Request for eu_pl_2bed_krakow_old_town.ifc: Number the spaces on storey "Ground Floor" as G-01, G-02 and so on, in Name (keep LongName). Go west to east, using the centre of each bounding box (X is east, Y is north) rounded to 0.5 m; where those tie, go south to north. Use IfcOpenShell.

First a look at what the model holds.

```python
import ifcopenshell
import ifcopenshell.util.element
import ifcopenshell.util.placement

model = ifcopenshell.open("eu_pl_2bed_krakow_old_town.ifc")
print(model.schema)
storey = next(s for s in model.by_type("IfcBuildingStorey") if s.Name == "Ground Floor")
spaces = [e for e in ifcopenshell.util.element.get_decomposition(storey) if e.is_a("IfcSpace")]
for e in sorted(spaces, key=lambda e: e.id()):
    origin = ifcopenshell.util.placement.get_local_placement(e.ObjectPlacement)[:3, 3]
    print(e.id(), e.Name, e.LongName, origin.round(2) + 0.0, sep=" | ")
```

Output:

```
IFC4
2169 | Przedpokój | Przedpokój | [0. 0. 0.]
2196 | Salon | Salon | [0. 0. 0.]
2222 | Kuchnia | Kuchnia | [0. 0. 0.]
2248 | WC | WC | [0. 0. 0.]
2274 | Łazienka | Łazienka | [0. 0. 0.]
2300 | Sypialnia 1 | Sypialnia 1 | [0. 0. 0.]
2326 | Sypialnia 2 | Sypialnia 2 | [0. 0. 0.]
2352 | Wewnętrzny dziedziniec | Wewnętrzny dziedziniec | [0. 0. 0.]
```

```python
import ifcopenshell
import ifcopenshell.geom
import ifcopenshell.util.element
import ifcopenshell.util.shape

model = ifcopenshell.open("eu_pl_2bed_krakow_old_town.ifc")
settings = ifcopenshell.geom.settings()
settings.set("use-world-coords", True)


def centre(element):
    shape = ifcopenshell.geom.create_shape(settings, element)
    return ifcopenshell.util.shape.get_bbox_centroid(shape.geometry)


storey = next(s for s in model.by_type("IfcBuildingStorey") if s.Name == "Ground Floor")
spaces = [e for e in ifcopenshell.util.element.get_decomposition(storey) if e.is_a("IfcSpace")]

# Insertion points can sit at a corner or the storey origin, so sort by the geometry (in metres).
centres = {e: centre(e) for e in spaces}
spaces.sort(key=lambda e: (round(centres[e][0] / 0.5), centres[e][1]))

for i, e in enumerate(spaces, start=1):
    number = f"G-{i:02d}"
    e.Name = number
    print(e.id(), number)

model.write("eu_pl_2bed_krakow_old_town_v2.ifc")
```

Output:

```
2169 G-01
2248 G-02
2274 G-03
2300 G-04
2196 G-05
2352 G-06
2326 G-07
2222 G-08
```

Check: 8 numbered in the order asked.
